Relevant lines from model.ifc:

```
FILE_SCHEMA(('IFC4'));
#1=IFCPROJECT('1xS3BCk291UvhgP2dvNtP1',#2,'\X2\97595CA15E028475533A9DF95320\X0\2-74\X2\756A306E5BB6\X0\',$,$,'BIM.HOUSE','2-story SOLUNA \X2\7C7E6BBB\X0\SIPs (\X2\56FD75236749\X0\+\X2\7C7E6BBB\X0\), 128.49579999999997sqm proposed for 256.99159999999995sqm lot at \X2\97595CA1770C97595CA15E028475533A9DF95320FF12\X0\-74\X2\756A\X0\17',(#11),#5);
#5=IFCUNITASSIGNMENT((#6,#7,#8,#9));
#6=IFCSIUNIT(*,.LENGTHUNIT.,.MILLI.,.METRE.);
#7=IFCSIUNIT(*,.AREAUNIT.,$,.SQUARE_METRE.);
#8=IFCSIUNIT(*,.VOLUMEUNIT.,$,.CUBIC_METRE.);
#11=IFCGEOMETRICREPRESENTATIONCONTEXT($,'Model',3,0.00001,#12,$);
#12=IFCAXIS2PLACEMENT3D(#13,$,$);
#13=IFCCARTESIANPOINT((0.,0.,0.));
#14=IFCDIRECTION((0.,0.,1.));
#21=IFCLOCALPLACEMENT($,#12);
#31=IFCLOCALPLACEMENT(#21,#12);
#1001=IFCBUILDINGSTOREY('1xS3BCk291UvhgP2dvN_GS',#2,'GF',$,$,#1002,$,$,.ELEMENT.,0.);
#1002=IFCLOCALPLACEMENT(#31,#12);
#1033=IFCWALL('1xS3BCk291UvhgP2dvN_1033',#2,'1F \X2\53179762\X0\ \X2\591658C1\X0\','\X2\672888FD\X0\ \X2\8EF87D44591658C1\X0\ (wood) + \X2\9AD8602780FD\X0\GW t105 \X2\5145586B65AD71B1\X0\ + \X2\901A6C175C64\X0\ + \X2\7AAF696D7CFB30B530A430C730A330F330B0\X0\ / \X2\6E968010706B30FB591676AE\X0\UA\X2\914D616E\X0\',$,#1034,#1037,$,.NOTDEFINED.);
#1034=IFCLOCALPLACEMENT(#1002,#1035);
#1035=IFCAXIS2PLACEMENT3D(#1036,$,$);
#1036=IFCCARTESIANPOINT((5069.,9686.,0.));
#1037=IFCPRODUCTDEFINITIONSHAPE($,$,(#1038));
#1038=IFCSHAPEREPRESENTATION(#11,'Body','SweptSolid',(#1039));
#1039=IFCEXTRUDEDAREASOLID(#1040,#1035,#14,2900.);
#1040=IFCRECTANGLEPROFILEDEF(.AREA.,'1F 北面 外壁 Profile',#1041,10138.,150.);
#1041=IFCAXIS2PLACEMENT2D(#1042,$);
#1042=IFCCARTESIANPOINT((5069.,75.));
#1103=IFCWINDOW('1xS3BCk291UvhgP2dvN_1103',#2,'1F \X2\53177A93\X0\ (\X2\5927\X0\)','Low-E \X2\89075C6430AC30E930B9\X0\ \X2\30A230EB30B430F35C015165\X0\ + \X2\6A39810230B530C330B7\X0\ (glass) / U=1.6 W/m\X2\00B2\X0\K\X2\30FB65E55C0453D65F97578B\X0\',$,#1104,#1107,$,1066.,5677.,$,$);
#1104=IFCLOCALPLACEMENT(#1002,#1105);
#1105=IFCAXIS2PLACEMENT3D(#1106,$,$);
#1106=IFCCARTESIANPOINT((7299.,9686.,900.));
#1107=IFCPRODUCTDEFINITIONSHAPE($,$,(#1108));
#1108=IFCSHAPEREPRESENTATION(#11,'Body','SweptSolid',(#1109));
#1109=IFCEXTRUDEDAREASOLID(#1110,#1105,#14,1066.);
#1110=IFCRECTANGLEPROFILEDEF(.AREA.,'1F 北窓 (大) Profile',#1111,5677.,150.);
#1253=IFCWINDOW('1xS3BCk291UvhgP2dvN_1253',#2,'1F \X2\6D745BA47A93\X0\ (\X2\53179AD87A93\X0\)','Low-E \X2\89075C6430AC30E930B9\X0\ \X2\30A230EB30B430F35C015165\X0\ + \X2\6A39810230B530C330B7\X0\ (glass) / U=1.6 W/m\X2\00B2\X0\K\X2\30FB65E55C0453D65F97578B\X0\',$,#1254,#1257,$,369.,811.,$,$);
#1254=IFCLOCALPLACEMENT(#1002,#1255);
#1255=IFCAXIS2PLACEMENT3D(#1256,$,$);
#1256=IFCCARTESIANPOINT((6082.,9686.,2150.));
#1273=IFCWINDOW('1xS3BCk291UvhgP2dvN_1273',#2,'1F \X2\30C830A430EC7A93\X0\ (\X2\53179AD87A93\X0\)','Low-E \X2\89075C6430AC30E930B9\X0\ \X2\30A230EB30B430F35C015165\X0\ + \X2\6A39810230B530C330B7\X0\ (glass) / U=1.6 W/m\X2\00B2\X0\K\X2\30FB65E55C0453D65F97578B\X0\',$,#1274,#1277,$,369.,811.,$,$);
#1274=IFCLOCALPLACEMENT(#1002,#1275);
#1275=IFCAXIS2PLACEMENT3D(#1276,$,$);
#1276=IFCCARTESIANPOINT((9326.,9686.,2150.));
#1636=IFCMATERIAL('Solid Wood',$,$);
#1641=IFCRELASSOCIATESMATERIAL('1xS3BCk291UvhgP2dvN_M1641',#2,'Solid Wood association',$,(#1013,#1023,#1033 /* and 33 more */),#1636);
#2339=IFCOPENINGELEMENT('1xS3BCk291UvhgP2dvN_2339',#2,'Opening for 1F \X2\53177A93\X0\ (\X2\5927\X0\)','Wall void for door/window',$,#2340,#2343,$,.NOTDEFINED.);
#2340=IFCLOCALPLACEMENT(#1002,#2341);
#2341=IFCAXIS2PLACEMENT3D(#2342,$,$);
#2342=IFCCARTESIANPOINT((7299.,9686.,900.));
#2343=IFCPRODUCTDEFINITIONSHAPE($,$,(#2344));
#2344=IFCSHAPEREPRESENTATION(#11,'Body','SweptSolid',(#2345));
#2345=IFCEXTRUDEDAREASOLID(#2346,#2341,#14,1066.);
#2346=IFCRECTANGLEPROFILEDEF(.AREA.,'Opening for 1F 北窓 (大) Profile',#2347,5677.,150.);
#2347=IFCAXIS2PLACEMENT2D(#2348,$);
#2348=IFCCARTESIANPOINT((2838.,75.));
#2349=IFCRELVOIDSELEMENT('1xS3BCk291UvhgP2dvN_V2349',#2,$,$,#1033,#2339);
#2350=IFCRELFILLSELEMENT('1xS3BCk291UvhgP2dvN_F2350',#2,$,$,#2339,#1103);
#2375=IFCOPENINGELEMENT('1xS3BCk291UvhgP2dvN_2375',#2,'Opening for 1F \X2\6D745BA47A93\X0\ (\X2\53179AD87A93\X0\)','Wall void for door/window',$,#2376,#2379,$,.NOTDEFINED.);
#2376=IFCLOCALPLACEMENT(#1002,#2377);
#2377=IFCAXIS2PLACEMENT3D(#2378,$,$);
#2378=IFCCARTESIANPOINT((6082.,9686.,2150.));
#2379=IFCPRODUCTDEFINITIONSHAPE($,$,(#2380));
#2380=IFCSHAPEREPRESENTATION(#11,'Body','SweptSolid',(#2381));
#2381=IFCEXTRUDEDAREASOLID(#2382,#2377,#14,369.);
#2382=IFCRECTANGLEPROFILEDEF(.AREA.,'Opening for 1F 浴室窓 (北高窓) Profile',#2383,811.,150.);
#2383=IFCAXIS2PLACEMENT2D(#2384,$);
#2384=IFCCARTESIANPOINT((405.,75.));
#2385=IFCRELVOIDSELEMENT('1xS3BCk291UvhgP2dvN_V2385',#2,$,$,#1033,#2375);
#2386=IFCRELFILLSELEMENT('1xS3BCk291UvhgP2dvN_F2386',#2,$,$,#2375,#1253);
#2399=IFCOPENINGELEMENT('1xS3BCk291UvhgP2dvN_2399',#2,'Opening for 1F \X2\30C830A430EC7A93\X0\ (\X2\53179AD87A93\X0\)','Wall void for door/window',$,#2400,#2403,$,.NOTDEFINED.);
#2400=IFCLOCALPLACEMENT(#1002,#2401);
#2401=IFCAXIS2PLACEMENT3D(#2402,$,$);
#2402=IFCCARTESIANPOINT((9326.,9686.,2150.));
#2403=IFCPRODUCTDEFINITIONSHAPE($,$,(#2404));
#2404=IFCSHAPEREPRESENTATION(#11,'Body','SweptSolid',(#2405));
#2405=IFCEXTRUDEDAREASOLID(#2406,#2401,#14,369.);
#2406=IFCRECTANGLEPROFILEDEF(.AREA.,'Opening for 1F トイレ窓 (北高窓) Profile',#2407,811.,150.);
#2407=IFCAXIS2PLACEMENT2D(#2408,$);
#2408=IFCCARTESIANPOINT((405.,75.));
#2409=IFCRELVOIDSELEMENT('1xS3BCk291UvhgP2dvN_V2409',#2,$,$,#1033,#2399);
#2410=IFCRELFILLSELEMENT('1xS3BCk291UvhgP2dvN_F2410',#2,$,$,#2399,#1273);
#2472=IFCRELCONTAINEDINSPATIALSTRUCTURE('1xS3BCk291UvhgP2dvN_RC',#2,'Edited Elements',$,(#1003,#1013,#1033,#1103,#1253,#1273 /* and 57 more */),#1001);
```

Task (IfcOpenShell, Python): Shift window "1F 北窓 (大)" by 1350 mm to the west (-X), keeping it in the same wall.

```python
import ifcopenshell
import ifcopenshell.api.geometry
import ifcopenshell.util.placement

model = ifcopenshell.open("model.ifc")

window = model.by_guid("1xS3BCk291UvhgP2dvN_1103")
opening = window.FillsVoids[0].RelatingOpeningElement
wall = opening.VoidsElements[0].RelatingBuildingElement

wall_matrix = ifcopenshell.util.placement.get_local_placement(wall.ObjectPlacement)
shift = wall_matrix[:3, 0] * -1350.0
before = ifcopenshell.util.placement.get_local_placement(window.ObjectPlacement)[:3, 3].copy()

# The window is not placed relative to its opening, so move both.
for product in (opening, window):
    matrix = ifcopenshell.util.placement.get_local_placement(product.ObjectPlacement)
    matrix[:3, 3] += shift
    ifcopenshell.api.geometry.edit_object_placement(model, product=product, matrix=matrix, is_si=False)

after = ifcopenshell.util.placement.get_local_placement(window.ObjectPlacement)[:3, 3]
print("window moved by", (after - before).round(3) + 0.0)

model.write("model-out.ifc")
```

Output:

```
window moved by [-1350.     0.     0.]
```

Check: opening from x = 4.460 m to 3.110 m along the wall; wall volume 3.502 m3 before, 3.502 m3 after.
